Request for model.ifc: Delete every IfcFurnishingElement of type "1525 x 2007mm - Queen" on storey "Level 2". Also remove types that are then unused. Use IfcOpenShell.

First a look at what the model holds.

```python
import ifcopenshell
import ifcopenshell.util.element

model = ifcopenshell.open("model.ifc")
print(model.schema)
storey = next(s for s in model.by_type("IfcBuildingStorey") if s.Name == "Level 2")
furniture = [e for e in ifcopenshell.util.element.get_decomposition(storey) if e.is_a("IfcFurnishingElement")]
seen = {}
for e in furniture:
    element_type = ifcopenshell.util.element.get_type(e)
    name = element_type.Name if element_type not in (None, e) else None
    seen[name] = seen.get(name, 0) + 1
for name, count in sorted(seen.items(), key=str):
    print(count, "x", name)
```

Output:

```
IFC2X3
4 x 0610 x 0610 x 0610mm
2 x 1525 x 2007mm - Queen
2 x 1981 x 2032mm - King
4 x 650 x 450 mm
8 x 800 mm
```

```python
import ifcopenshell
import ifcopenshell.api.root
import ifcopenshell.util.element

model = ifcopenshell.open("model.ifc")

storey = next(s for s in model.by_type("IfcBuildingStorey") if s.Name == "Level 2")
furniture = [e for e in ifcopenshell.util.element.get_decomposition(storey) if e.is_a("IfcFurnishingElement")]
targets = [e for e in furniture if (t := ifcopenshell.util.element.get_type(e)) not in (None, e) and t.Name == "1525 x 2007mm - Queen"]
types = {ifcopenshell.util.element.get_type(e) for e in targets} - {None, *targets}

for e in targets:
    ifcopenshell.api.root.remove_product(model, product=e)
print(len(targets), "removed")

unused = [t for t in types if not ifcopenshell.util.element.get_types(t)]
for t in unused:
    ifcopenshell.api.root.remove_product(model, product=t)
print(len(unused), "unused types removed")

model.write("model_rev.ifc")
```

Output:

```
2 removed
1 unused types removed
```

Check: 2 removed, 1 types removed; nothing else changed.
